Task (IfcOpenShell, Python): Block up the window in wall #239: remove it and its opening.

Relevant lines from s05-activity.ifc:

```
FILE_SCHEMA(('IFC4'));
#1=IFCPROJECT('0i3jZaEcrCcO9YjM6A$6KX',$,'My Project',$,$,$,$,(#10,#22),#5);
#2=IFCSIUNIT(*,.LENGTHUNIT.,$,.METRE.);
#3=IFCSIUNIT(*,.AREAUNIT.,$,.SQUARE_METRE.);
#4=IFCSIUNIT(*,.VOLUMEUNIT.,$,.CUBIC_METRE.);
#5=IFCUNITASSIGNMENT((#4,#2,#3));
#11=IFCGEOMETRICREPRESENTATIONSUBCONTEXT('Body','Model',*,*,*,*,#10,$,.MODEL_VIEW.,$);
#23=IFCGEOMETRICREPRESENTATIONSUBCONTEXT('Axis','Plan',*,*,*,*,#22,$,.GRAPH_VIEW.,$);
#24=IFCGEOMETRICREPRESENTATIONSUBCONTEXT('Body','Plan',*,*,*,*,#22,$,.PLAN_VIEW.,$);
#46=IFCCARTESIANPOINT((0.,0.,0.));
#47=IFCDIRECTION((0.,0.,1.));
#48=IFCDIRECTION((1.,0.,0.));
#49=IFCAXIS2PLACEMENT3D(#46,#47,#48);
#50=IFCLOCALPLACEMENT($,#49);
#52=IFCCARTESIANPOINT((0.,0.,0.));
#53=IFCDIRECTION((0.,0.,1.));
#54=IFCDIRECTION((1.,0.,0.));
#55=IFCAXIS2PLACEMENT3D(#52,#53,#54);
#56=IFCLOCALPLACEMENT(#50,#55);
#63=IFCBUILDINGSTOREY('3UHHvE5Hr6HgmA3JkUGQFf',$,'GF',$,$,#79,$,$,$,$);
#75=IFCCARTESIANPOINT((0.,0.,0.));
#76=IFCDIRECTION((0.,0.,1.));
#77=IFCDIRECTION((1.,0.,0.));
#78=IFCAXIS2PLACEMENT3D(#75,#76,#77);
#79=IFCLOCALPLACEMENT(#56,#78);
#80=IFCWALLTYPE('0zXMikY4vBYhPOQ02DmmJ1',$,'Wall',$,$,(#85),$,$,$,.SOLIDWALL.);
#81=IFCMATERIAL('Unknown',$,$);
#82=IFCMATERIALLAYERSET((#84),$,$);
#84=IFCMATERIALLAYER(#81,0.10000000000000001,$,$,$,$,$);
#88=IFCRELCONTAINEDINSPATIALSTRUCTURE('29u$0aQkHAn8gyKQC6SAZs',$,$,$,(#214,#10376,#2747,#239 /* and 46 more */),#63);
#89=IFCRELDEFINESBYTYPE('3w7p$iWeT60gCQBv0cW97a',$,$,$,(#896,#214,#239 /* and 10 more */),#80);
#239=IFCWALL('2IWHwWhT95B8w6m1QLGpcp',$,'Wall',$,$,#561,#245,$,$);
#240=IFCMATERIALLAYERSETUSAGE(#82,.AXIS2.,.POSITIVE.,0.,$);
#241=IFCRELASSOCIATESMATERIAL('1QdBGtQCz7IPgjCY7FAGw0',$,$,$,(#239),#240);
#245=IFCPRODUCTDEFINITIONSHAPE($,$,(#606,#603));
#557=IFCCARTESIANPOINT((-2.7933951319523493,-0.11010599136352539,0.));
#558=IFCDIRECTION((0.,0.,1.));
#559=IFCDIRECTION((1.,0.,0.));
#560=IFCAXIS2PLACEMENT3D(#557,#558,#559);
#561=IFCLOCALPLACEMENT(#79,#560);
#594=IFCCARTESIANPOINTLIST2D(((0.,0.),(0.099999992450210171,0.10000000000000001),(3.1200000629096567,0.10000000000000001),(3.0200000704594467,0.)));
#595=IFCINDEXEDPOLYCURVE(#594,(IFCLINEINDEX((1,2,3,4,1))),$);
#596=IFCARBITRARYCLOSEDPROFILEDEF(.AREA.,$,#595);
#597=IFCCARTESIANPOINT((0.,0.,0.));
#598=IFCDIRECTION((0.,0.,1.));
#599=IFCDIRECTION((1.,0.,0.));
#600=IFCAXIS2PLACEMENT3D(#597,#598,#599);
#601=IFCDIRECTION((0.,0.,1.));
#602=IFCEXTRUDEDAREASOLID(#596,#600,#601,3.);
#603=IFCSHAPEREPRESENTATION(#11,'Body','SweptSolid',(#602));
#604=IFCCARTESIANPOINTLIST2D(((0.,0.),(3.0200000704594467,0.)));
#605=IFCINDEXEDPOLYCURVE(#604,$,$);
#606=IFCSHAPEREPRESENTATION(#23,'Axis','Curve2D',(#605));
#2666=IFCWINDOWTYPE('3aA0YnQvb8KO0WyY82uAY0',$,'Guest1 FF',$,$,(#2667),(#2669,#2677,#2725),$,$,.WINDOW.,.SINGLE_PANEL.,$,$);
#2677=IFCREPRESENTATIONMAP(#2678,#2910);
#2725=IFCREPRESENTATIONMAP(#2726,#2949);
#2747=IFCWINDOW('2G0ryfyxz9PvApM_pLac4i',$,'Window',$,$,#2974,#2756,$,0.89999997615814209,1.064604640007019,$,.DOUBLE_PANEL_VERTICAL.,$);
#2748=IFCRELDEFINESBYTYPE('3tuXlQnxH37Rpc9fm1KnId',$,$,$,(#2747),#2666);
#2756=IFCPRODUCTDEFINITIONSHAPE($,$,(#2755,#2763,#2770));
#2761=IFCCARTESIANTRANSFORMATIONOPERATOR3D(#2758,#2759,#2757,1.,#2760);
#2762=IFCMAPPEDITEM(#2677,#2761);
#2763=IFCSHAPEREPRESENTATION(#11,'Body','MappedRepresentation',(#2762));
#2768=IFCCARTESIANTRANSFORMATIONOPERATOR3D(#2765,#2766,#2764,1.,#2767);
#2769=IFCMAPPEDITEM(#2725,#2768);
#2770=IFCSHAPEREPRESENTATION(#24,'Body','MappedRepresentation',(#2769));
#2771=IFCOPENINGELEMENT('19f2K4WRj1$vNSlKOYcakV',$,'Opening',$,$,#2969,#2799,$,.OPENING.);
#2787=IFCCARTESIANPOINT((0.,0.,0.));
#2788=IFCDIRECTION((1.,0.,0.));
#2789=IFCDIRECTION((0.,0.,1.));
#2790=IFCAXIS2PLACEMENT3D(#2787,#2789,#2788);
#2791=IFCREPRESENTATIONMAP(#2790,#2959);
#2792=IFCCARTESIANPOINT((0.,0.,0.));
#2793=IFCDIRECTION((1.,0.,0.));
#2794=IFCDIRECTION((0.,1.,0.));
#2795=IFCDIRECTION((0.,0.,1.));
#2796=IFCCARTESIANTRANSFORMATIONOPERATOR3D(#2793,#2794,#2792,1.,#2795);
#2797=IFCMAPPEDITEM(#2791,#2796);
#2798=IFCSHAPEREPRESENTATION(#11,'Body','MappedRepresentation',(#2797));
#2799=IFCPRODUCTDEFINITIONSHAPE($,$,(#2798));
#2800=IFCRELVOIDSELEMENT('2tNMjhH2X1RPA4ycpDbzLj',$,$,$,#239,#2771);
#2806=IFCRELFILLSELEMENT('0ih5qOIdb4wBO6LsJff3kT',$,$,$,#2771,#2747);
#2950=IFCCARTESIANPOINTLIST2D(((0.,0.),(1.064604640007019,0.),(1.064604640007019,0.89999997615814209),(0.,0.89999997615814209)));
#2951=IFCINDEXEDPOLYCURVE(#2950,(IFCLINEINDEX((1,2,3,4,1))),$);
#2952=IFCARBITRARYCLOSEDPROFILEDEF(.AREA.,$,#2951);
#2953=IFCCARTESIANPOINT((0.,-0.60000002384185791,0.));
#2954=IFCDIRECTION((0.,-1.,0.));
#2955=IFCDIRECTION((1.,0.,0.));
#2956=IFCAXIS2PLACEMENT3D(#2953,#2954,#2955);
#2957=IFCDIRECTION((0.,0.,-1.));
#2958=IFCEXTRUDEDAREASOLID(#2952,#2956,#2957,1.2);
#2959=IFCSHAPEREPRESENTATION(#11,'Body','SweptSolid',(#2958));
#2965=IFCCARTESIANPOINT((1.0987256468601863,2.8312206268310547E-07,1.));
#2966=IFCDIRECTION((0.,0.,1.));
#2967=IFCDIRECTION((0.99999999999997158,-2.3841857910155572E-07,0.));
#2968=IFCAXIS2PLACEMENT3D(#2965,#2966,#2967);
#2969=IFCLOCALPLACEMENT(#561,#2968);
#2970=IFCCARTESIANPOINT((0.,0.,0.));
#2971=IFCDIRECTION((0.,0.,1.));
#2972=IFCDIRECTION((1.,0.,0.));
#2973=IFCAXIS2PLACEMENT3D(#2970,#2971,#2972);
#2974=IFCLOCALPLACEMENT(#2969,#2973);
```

```python
import ifcopenshell
import ifcopenshell.api.feature
import ifcopenshell.api.root
import ifcopenshell.geom
import ifcopenshell.util.shape

model = ifcopenshell.open("s05-activity.ifc")
settings = ifcopenshell.geom.settings()


def volume(element):
    """Net volume in cubic metres, openings subtracted."""
    shape = ifcopenshell.geom.create_shape(settings, element)
    return ifcopenshell.util.shape.get_volume(shape.geometry)


window = model.by_guid("2G0ryfyxz9PvApM_pLac4i")
opening = window.FillsVoids[0].RelatingOpeningElement
wall = opening.VoidsElements[0].RelatingBuildingElement
before = volume(wall)

ifcopenshell.api.root.remove_product(model, product=window)
ifcopenshell.api.feature.remove_feature(model, feature=opening)

after = volume(wall)

print(f"wall volume {before:.3f} -> {after:.3f} m3")

model.write("s05-activity_edited.ifc")
```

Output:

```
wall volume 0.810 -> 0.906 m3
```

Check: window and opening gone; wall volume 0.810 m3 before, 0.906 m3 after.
